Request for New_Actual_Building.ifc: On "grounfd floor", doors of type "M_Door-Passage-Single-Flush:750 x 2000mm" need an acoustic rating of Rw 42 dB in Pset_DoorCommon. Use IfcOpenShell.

First a look at what the model holds.

```python
import ifcopenshell
import ifcopenshell.util.element

model = ifcopenshell.open("New_Actual_Building.ifc")
print(model.schema)
storey = next(s for s in model.by_type("IfcBuildingStorey") if s.Name == "grounfd floor")
doors = [e for e in ifcopenshell.util.element.get_decomposition(storey) if e.is_a("IfcDoor")]
seen = {}
for e in doors:
    element_type = ifcopenshell.util.element.get_type(e)
    key = (element_type.Name if element_type != e and element_type else None, ifcopenshell.util.element.get_pset(e, "Pset_DoorCommon", "AcousticRating"))
    seen[key] = seen.get(key, 0) + 1
for (name, value), count in sorted(seen.items(), key=str):
    print(count, "x", name, "|", value)
```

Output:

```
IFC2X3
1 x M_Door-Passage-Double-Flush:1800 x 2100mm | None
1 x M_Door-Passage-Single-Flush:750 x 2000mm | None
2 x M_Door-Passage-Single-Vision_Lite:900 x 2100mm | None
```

```python
import ifcopenshell
import ifcopenshell.api.pset
import ifcopenshell.util.element

model = ifcopenshell.open("New_Actual_Building.ifc")

storey = next(s for s in model.by_type("IfcBuildingStorey") if s.Name == "grounfd floor")
doors = [e for e in ifcopenshell.util.element.get_decomposition(storey) if e.is_a("IfcDoor")]

count = 0
for e in doors:
    element_type = ifcopenshell.util.element.get_type(e)
    if element_type in (None, e) or element_type.Name != "M_Door-Passage-Single-Flush:750 x 2000mm":
        continue
    # add_pset returns the element's existing set when there is one.
    pset = ifcopenshell.api.pset.add_pset(model, product=e, name="Pset_DoorCommon")
    ifcopenshell.api.pset.edit_pset(model, pset=pset, properties={"AcousticRating": "Rw 42 dB"})
    count += 1

print(count, "doors updated")

model.write("New_Actual_Building_updated.ifc")
```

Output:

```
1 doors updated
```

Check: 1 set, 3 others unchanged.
